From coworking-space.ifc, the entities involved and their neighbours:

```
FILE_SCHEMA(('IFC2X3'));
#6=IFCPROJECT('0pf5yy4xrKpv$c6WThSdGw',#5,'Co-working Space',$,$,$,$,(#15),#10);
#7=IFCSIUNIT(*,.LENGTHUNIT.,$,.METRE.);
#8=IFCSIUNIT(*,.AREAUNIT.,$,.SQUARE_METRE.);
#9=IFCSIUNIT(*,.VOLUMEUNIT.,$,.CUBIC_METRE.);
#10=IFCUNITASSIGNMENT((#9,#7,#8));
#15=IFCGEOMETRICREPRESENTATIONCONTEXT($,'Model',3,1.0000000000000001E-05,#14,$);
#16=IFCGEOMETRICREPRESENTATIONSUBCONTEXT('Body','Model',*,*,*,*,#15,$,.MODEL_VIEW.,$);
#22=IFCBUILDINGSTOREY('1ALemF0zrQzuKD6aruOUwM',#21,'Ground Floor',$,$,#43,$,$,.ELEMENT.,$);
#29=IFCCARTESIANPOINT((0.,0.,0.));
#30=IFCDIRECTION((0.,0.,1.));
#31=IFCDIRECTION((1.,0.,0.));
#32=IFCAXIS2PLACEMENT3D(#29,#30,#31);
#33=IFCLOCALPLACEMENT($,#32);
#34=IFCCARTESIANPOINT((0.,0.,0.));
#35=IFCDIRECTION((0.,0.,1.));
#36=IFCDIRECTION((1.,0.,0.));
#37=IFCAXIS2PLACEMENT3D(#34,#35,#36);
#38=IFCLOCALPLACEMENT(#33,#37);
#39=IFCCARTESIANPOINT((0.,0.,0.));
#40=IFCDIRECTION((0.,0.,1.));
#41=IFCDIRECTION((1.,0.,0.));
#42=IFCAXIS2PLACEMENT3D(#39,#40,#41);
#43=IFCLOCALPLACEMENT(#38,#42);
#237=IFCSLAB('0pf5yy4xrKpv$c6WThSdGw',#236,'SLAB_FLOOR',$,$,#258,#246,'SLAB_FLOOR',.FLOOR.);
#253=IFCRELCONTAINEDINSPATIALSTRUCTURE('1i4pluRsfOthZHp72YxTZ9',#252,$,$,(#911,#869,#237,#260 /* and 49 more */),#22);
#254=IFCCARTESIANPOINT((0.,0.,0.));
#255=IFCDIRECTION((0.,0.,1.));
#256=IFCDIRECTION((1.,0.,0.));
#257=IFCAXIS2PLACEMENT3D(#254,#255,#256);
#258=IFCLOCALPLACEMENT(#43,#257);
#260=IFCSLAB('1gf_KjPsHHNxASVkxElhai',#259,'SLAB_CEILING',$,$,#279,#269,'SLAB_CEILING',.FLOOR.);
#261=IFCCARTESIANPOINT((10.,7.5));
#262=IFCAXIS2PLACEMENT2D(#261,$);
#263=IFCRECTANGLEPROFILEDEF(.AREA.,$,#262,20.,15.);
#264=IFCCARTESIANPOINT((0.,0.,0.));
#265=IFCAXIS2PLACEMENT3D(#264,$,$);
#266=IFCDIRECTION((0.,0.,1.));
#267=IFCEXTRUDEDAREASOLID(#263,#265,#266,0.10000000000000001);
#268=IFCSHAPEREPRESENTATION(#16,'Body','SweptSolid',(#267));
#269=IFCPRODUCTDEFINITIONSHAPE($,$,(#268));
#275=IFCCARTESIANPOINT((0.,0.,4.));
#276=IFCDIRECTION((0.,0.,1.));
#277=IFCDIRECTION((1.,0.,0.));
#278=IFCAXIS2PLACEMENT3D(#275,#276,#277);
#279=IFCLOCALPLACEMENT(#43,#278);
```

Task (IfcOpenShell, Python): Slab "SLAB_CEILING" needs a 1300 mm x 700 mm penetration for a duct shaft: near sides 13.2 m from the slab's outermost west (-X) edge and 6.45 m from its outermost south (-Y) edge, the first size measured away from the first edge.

```python
import numpy as np
import ifcopenshell
import ifcopenshell.api.feature
import ifcopenshell.api.geometry
import ifcopenshell.api.root
import ifcopenshell.geom
import ifcopenshell.util.placement
import ifcopenshell.util.representation
import ifcopenshell.util.shape
import ifcopenshell.util.unit

model = ifcopenshell.open("coworking-space.ifc")
unit_scale = ifcopenshell.util.unit.calculate_unit_scale(model)
settings = ifcopenshell.geom.settings()


def volume(element):
    """Net volume in cubic metres, openings subtracted."""
    shape = ifcopenshell.geom.create_shape(settings, element)
    return ifcopenshell.util.shape.get_volume(shape.geometry)


slab = model.by_id(260)
before = volume(slab)

# Extent in the slab's own axes, in metres. The edges named are its -X and -Y sides.
slab_shape = ifcopenshell.geom.create_shape(settings, slab)
vertices = ifcopenshell.util.shape.get_vertices(slab_shape.geometry)
x_min, y_min, bottom = vertices.min(axis=0)
top = vertices[:, 2].max()

opening = ifcopenshell.api.root.create_entity(model, ifc_class="IfcOpeningElement", name="Duct shaft opening")
context = ifcopenshell.util.representation.get_context(model, "Model", "Body", "MODEL_VIEW")
width, depth = 1.3, 0.7
outline = [(0.0, 0.0), (width, 0.0), (width, depth), (0.0, depth), (0.0, 0.0)]
# Overshoot both faces by 50 mm so the cut is clean.
shape = ifcopenshell.api.geometry.add_slab_representation(
    model, context=context, depth=top - bottom + 0.1, polyline=outline
)
ifcopenshell.api.geometry.assign_representation(model, product=opening, representation=shape)

matrix = ifcopenshell.util.placement.get_local_placement(slab.ObjectPlacement)
matrix[:, 3] = matrix @ np.append(np.array([x_min + 13.2, y_min + 6.45, bottom - 0.05]) / unit_scale, 1.0)
ifcopenshell.api.geometry.edit_object_placement(model, product=opening, matrix=matrix, is_si=False)
ifcopenshell.api.feature.add_feature(model, feature=opening, element=slab)

after = volume(slab)

print(f"slab volume {before:.3f} -> {after:.3f} m3")

model.write("coworking-space_rev.ifc")
```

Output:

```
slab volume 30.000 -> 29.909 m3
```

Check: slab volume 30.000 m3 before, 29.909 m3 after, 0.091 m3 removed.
